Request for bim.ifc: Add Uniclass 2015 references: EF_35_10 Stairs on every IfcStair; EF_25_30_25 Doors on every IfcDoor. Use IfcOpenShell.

First a look at what the model holds.

```python
import ifcopenshell

model = ifcopenshell.open("bim.ifc")
print(model.schema)
print("classifications:", [c.Name for c in model.by_type("IfcClassification")])
for ifc_class in ("IfcDoor", "IfcRoof", "IfcStair", "IfcWall", "IfcWindow"):
    print(ifc_class, len(model.by_type(ifc_class)))
```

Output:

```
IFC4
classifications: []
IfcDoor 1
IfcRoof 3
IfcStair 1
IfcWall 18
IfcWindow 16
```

```python
import ifcopenshell
import ifcopenshell.api.classification

model = ifcopenshell.open("bim.ifc")

system = ifcopenshell.api.classification.add_classification(model, classification="Uniclass 2015")

codes = {
    "IfcStair": ("EF_35_10", "Stairs"),
    "IfcDoor": ("EF_25_30_25", "Doors"),
}
for ifc_class, (code, name) in codes.items():
    products = model.by_type(ifc_class)
    ifcopenshell.api.classification.add_reference(
        model, products=products, classification=system, identification=code, name=name
    )
    print(code, len(products))

model.write("bim-out.ifc")
```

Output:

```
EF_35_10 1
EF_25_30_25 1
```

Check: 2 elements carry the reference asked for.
